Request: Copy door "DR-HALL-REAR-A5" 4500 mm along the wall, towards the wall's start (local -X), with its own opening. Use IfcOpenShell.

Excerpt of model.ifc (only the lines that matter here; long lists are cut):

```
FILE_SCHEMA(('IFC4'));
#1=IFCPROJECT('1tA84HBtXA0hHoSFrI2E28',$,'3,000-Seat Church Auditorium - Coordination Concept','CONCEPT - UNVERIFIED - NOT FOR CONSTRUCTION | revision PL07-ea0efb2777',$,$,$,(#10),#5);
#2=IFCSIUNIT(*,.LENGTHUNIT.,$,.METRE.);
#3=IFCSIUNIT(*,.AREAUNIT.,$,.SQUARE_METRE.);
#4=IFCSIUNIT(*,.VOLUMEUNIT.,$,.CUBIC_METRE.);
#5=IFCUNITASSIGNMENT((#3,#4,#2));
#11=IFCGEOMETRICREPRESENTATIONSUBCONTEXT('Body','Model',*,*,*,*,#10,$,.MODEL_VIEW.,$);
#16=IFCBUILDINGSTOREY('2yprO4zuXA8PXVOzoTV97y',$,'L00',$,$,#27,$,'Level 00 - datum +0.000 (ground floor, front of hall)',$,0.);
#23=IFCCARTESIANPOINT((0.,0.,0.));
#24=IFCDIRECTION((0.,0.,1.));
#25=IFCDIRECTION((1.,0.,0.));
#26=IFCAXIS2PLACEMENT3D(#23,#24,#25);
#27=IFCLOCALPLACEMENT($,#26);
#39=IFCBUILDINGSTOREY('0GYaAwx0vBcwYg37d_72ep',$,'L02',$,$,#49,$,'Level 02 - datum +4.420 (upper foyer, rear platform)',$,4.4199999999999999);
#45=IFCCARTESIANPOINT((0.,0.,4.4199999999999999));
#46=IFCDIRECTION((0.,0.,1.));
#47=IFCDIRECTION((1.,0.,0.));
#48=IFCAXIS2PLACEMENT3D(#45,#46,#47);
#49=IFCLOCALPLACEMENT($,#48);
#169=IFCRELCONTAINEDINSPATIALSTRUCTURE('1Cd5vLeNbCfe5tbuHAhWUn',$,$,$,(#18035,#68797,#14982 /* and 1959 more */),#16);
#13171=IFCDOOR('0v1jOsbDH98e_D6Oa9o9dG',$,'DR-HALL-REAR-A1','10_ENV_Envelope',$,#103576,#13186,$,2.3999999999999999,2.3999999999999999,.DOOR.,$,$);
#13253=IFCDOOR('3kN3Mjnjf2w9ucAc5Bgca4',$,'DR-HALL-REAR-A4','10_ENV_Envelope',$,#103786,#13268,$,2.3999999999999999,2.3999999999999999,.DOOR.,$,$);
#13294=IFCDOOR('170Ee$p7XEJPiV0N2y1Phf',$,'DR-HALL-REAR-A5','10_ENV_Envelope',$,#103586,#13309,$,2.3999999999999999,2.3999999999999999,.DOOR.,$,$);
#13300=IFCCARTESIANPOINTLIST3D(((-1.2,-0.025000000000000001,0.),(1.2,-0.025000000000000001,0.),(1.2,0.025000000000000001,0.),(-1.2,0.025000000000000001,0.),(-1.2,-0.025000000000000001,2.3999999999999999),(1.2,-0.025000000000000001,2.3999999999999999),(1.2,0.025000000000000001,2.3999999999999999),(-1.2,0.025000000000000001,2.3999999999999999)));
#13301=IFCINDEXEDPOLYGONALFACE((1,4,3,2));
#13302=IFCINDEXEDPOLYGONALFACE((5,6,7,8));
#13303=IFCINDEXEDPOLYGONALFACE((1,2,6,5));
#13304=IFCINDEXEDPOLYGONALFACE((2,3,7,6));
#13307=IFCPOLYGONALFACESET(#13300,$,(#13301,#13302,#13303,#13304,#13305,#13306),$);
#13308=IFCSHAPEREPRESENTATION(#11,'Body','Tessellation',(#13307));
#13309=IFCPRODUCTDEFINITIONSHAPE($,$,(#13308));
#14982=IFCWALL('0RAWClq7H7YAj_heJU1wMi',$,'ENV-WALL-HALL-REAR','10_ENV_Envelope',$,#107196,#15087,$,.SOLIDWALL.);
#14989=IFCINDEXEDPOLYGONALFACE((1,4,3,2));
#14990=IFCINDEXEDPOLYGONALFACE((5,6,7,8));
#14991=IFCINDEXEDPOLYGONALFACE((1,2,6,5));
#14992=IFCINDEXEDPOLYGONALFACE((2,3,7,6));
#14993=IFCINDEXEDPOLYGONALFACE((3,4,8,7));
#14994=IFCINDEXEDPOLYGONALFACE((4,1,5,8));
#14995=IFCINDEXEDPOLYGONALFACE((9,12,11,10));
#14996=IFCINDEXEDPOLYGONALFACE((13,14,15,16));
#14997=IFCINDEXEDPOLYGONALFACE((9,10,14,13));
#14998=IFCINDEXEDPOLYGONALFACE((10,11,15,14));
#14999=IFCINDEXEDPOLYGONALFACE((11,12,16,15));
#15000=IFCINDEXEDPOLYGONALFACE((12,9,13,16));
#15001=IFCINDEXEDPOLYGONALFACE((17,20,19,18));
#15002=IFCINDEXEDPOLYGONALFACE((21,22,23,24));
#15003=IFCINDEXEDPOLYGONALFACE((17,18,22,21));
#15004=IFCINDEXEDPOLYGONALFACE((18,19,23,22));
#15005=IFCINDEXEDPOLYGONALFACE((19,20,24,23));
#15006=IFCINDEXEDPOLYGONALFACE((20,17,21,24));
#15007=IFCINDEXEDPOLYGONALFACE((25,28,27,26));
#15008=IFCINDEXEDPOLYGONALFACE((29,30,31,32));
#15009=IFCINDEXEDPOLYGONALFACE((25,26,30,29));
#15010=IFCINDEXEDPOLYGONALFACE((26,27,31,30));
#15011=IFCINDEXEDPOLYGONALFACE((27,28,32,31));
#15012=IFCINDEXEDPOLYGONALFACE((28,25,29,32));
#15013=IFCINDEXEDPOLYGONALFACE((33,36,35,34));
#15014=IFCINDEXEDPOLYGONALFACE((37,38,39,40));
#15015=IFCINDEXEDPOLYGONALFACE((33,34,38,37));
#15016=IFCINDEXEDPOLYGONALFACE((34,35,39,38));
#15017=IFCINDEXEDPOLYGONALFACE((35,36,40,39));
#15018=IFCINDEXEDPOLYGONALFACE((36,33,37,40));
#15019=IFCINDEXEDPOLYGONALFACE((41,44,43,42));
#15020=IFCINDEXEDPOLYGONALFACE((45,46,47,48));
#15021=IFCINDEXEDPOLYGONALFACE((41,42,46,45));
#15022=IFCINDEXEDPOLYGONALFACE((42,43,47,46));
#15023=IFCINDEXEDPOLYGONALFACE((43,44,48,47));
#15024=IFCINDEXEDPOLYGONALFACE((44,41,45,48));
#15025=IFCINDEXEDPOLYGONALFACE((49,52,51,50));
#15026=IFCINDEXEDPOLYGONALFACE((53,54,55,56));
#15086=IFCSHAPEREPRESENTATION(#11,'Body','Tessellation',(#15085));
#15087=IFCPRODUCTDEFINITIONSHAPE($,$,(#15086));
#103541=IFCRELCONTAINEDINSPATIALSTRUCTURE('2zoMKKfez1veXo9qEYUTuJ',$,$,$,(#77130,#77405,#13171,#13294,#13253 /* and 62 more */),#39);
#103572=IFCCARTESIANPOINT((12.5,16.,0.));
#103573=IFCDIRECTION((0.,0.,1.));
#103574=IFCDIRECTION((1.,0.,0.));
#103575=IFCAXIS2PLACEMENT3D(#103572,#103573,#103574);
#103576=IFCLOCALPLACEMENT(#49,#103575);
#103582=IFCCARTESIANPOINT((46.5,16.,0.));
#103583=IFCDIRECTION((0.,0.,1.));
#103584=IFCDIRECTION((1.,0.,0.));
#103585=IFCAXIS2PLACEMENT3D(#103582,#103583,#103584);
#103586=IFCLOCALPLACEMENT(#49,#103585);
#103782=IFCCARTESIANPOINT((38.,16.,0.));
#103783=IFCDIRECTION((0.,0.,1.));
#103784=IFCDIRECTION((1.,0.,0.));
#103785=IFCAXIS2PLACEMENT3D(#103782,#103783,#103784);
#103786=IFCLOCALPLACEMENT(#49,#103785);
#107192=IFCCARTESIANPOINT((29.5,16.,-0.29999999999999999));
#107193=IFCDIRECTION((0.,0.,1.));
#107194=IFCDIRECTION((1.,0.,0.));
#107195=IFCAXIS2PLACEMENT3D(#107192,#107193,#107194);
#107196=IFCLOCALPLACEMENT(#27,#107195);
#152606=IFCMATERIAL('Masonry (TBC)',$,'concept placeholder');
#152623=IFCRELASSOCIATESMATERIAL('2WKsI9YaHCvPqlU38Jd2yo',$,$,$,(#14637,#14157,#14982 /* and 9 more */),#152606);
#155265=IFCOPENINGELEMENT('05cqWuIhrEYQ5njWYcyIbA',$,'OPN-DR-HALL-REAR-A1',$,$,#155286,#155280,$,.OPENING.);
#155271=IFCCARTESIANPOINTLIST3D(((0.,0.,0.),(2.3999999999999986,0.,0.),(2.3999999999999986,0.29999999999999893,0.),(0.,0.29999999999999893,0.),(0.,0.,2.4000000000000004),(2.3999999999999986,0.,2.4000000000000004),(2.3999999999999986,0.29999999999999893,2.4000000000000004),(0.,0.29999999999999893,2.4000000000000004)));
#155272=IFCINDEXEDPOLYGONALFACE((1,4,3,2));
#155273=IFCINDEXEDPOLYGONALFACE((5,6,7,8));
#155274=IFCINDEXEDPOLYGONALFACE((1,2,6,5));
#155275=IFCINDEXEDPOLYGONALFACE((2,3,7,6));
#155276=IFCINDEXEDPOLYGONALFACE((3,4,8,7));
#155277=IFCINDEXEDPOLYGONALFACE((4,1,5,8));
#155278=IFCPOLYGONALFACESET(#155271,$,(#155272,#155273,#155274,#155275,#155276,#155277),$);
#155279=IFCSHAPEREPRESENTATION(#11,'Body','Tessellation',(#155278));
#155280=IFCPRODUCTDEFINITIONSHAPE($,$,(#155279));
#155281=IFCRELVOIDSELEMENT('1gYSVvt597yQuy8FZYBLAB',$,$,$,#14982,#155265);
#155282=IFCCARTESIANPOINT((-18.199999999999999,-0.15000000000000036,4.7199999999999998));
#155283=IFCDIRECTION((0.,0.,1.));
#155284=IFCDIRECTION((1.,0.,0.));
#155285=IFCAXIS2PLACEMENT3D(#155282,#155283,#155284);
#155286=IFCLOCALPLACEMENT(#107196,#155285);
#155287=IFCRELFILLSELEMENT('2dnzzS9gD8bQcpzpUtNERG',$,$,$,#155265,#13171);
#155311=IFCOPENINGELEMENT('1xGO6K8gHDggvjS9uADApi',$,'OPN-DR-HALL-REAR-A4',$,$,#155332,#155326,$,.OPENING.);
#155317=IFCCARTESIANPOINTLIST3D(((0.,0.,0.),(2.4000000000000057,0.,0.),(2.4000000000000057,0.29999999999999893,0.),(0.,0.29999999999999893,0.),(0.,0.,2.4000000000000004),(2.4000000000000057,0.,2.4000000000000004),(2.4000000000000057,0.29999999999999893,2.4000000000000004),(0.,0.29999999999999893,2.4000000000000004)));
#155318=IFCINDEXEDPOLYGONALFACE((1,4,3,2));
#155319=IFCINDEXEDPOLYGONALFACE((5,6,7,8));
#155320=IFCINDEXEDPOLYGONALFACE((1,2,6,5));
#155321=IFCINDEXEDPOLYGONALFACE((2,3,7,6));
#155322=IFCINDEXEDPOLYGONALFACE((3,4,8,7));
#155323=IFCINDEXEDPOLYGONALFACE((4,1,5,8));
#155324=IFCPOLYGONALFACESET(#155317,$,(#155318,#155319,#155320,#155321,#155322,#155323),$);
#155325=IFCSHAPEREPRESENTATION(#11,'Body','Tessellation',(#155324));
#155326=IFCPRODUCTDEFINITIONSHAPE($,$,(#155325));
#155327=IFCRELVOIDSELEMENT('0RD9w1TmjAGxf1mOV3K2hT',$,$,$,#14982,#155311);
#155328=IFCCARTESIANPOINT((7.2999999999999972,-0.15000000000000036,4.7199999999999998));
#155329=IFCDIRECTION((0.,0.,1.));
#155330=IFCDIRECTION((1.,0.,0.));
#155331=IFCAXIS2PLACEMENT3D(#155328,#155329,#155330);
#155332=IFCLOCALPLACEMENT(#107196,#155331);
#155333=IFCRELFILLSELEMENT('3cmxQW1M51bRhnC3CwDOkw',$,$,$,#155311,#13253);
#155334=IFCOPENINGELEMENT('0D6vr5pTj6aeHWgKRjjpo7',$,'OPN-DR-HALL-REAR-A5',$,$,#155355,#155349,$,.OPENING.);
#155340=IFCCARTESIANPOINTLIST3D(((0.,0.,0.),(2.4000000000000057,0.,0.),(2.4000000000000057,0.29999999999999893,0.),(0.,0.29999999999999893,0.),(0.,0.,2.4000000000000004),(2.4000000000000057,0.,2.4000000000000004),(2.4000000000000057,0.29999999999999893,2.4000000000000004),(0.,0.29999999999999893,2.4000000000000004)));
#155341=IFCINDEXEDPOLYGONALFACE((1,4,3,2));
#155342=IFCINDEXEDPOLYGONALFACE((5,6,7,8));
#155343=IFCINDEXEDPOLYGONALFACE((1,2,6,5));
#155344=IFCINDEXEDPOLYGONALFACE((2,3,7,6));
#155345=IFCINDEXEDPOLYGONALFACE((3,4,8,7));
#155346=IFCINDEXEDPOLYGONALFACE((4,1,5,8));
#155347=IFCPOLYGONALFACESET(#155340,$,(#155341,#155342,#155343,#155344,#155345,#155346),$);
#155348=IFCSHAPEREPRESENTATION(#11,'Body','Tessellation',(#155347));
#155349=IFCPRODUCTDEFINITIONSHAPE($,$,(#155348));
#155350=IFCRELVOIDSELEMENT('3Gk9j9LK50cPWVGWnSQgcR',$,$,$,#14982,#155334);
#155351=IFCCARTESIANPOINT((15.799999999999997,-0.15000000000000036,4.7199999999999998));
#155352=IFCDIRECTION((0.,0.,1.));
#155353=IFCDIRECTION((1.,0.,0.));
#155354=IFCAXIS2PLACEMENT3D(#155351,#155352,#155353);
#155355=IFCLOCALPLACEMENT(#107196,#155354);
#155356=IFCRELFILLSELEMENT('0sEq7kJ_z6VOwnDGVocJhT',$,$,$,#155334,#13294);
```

```python
import ifcopenshell
import ifcopenshell.api.feature
import ifcopenshell.api.geometry
import ifcopenshell.api.root
import ifcopenshell.geom
import ifcopenshell.util.element
import ifcopenshell.util.placement
import ifcopenshell.util.shape
import ifcopenshell.util.unit

model = ifcopenshell.open("model.ifc")
unit_scale = ifcopenshell.util.unit.calculate_unit_scale(model)
settings = ifcopenshell.geom.settings()


def volume(element):
    """Net volume in cubic metres, openings subtracted."""
    shape = ifcopenshell.geom.create_shape(settings, element)
    return ifcopenshell.util.shape.get_volume(shape.geometry)


door = model.by_guid("170Ee$p7XEJPiV0N2y1Phf")
opening = door.FillsVoids[0].RelatingOpeningElement
wall = opening.VoidsElements[0].RelatingBuildingElement
before = volume(wall)
shift = ifcopenshell.util.placement.get_local_placement(wall.ObjectPlacement)[:3, 0] * -4.5 / unit_scale

# copy_class copies the void relationship, type, container and properties, but no geometry.
new_opening = ifcopenshell.api.root.copy_class(model, product=opening)
new_opening.Representation = ifcopenshell.util.element.copy_deep(
    model, opening.Representation, exclude=["IfcGeometricRepresentationContext", "IfcRepresentationMap"]
)
new_door = ifcopenshell.api.root.copy_class(model, product=door)
new_door.Representation = ifcopenshell.util.element.copy_deep(
    model, door.Representation, exclude=["IfcGeometricRepresentationContext", "IfcRepresentationMap"]
)
ifcopenshell.api.feature.add_filling(model, opening=new_opening, element=new_door)

for old, new in ((opening, new_opening), (door, new_door)):
    matrix = ifcopenshell.util.placement.get_local_placement(old.ObjectPlacement)
    matrix[:3, 3] += shift
    ifcopenshell.api.geometry.edit_object_placement(model, product=new, matrix=matrix, is_si=False)

after = volume(wall)

print(f"wall volume {before:.3f} -> {after:.3f} m3")

model.write("model_v2.ifc")
```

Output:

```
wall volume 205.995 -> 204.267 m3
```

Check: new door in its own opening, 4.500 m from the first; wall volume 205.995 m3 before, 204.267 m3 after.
